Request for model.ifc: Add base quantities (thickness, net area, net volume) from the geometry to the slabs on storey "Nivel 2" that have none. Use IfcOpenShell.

First a look at what the model holds.

```python
import ifcopenshell
import ifcopenshell.util.element
import ifcopenshell.util.unit

model = ifcopenshell.open("model.ifc")
print(model.schema)
for unit_type in ("LENGTHUNIT", "AREAUNIT", "VOLUMEUNIT"):
    print(unit_type, ifcopenshell.util.unit.calculate_unit_scale(model, unit_type))
storey = next(s for s in model.by_type("IfcBuildingStorey") if s.Name == "Nivel 2")
slabs = [e for e in ifcopenshell.util.element.get_decomposition(storey) if e.is_a("IfcSlab")]
for e in sorted(slabs, key=lambda e: e.id()):
    print(e.id(), e.is_a(), e.Name, list(ifcopenshell.util.element.get_psets(e, qtos_only=True)), sep=" | ")
```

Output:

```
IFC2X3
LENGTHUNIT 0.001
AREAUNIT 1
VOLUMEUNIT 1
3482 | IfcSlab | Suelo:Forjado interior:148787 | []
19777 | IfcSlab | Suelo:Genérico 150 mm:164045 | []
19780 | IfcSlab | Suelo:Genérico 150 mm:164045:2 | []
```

```python
import ifcopenshell
import ifcopenshell.api.pset
import ifcopenshell.geom
import ifcopenshell.util.element
import ifcopenshell.util.shape
import ifcopenshell.util.unit

model = ifcopenshell.open("model.ifc")
unit_scale = ifcopenshell.util.unit.calculate_unit_scale(model)
area_scale = ifcopenshell.util.unit.calculate_unit_scale(model, "AREAUNIT")
volume_scale = ifcopenshell.util.unit.calculate_unit_scale(model, "VOLUMEUNIT")
settings = ifcopenshell.geom.settings()

storey = next(s for s in model.by_type("IfcBuildingStorey") if s.Name == "Nivel 2")
slabs = [e for e in ifcopenshell.util.element.get_decomposition(storey) if e.is_a("IfcSlab")]

for e in sorted(slabs, key=lambda e: e.id()):
    if ifcopenshell.util.element.get_psets(e, qtos_only=True, should_inherit=False):
        continue
    # Geometry comes back in metres, in the element's own axes.
    shape = ifcopenshell.geom.create_shape(settings, e)
    values = {
        "Width": ifcopenshell.util.shape.get_z(shape.geometry) / unit_scale,
        "NetArea": ifcopenshell.util.shape.get_footprint_area(shape.geometry) / area_scale,
        "NetVolume": ifcopenshell.util.shape.get_volume(shape.geometry) / volume_scale,
    }
    qto = ifcopenshell.api.pset.add_qto(model, product=e, name="BaseQuantities")
    ifcopenshell.api.pset.edit_qto(model, qto=qto, properties=values)
    print(e.id(), {k: round(v, 3) for k, v in values.items()})

model.write("model_v2.ifc")
```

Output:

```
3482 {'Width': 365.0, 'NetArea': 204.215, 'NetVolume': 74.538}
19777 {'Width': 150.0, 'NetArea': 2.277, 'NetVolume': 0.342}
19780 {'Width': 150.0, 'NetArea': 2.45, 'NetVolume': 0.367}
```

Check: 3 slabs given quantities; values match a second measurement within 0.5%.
